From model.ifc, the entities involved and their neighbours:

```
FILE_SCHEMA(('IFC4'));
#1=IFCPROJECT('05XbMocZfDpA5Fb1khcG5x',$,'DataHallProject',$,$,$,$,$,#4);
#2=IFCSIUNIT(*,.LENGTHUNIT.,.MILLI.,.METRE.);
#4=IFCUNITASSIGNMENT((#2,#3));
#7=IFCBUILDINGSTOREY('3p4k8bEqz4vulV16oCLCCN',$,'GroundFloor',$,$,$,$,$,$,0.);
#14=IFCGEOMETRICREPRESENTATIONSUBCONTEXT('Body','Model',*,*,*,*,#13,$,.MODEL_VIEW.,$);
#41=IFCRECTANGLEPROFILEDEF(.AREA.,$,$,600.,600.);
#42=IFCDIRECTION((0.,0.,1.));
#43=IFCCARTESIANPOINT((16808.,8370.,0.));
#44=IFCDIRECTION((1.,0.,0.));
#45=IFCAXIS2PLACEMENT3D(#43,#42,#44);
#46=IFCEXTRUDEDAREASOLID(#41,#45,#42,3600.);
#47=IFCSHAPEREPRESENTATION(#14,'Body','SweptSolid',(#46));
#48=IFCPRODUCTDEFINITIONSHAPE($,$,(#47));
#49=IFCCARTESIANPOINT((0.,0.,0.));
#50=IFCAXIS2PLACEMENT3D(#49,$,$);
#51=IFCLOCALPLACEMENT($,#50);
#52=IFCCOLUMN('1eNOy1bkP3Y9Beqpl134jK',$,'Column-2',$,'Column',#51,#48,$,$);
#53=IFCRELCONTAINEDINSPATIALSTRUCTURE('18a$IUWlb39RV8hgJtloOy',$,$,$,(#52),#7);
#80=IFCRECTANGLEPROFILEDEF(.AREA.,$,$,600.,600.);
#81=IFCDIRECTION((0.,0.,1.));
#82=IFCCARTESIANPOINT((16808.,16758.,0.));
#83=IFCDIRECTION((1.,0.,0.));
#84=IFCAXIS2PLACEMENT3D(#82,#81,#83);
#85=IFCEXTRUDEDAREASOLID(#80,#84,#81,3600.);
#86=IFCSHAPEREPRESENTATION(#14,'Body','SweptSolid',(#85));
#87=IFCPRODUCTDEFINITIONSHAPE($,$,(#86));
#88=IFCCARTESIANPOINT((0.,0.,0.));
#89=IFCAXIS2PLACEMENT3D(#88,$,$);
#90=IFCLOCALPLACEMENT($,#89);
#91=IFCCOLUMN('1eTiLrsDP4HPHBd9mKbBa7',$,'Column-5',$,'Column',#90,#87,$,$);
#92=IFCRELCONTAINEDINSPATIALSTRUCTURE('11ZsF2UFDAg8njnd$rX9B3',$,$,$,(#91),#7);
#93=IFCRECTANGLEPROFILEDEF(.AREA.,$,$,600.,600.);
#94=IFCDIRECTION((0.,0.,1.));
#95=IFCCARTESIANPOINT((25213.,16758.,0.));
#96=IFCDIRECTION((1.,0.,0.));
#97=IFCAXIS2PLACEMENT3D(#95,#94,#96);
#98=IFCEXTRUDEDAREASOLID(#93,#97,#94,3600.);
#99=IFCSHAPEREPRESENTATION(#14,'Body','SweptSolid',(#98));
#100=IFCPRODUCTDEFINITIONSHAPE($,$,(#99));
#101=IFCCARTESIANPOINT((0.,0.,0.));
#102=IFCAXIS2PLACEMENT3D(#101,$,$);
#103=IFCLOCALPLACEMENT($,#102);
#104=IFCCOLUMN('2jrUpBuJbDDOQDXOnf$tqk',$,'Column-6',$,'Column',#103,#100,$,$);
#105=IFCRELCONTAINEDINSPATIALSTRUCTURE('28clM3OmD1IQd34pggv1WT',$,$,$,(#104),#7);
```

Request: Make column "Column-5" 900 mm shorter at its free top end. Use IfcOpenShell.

```python
import ifcopenshell
import ifcopenshell.util.representation
import ifcopenshell.util.unit

model = ifcopenshell.open("model.ifc")
unit_scale = ifcopenshell.util.unit.calculate_unit_scale(model)

member = model.by_id(91)
change = -0.9 / unit_scale

# The extrusion runs towards the end named, so only its depth changes.
body = ifcopenshell.util.representation.get_representation(member, "Model", "Body")
solid = body.Items[0]
old_length = solid.Depth
solid.Depth += change

print(f"length {old_length:g} -> {solid.Depth:g}")

model.write("model-out.ifc")
```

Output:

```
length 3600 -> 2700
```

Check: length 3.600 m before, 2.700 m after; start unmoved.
